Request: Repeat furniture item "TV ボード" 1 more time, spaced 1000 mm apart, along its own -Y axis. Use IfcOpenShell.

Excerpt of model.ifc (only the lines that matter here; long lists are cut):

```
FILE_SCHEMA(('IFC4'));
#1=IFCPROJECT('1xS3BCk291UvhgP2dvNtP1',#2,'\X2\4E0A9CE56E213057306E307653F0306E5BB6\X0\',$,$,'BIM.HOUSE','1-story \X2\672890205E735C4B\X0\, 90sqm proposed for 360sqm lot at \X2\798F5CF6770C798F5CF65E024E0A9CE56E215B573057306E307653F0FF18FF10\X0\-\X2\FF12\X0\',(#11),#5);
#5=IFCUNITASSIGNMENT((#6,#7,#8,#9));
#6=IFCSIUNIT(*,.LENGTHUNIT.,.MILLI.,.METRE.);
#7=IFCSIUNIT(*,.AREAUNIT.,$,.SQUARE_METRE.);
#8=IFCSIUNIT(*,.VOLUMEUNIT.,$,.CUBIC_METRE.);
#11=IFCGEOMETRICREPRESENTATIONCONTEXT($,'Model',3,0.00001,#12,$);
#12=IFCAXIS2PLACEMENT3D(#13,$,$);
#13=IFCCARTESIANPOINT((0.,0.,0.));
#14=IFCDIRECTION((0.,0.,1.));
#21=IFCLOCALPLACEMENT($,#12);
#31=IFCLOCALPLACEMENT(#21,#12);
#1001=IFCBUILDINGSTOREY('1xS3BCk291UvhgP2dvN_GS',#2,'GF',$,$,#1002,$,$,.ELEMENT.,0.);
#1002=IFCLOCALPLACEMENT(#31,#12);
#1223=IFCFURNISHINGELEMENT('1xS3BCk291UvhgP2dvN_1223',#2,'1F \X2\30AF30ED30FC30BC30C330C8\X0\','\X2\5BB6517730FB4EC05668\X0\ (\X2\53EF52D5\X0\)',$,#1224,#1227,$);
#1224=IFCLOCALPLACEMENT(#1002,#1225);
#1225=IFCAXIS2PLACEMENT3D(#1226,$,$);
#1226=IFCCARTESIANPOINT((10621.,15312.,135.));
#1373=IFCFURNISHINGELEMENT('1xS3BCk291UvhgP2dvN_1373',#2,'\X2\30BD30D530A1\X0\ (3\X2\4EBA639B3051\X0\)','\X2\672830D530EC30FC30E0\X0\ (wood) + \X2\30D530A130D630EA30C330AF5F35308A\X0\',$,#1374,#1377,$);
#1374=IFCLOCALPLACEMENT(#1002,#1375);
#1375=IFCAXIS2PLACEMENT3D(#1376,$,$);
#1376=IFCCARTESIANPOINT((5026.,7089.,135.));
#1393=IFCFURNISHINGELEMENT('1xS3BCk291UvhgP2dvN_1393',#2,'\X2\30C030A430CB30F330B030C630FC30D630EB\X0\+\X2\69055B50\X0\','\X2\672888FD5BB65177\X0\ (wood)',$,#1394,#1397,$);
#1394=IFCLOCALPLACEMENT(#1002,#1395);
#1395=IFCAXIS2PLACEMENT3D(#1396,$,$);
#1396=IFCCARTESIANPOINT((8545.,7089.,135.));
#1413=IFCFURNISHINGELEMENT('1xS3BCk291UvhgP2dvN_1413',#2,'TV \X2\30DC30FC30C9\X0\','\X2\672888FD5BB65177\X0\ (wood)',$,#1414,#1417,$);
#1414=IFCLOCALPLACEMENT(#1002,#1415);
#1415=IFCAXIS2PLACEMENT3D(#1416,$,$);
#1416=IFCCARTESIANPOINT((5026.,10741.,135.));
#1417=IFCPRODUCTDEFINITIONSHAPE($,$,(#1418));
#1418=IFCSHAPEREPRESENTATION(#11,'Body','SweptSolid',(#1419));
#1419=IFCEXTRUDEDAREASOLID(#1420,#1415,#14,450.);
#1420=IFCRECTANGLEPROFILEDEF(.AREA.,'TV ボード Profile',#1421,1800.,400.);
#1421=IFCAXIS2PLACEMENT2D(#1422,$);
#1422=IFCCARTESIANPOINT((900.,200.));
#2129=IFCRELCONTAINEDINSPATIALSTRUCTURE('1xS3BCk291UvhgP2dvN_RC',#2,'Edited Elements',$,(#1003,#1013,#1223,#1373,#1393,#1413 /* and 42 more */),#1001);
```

```python
import ifcopenshell
import ifcopenshell.api.geometry
import ifcopenshell.api.root
import ifcopenshell.util.element
import ifcopenshell.util.placement

model = ifcopenshell.open("model.ifc")


def reuse_history(source, copy):
    """copy_class also copies each property set's owner history, people and application; keep the originals."""
    for rel in copy.IsDefinedBy:
        if rel.is_a("IfcRelDefinesByProperties") and (history := rel.RelatingPropertyDefinition.OwnerHistory):
            rel.RelatingPropertyDefinition.OwnerHistory = source.OwnerHistory
            ifcopenshell.util.element.remove_deep2(model, history)


source = model.by_guid("1xS3BCk291UvhgP2dvN_1413")
base = ifcopenshell.util.placement.get_local_placement(source.ObjectPlacement)
step = -base[:3, 1] * 1000.0

for i in range(1, 2):
    copy = ifcopenshell.api.root.copy_class(model, product=source)
    copy.Representation = ifcopenshell.util.element.copy_deep(
        model, source.Representation, exclude=["IfcGeometricRepresentationContext", "IfcRepresentationMap"]
    )
    reuse_history(source, copy)
    matrix = base.copy()
    matrix[:3, 3] += i * step
    print("added at", matrix[:3, 3].round(3) + 0.0)
    ifcopenshell.api.geometry.edit_object_placement(model, product=copy, matrix=matrix, is_si=False)

model.write("model_v2.ifc")
```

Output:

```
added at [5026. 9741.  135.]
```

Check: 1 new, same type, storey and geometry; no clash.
